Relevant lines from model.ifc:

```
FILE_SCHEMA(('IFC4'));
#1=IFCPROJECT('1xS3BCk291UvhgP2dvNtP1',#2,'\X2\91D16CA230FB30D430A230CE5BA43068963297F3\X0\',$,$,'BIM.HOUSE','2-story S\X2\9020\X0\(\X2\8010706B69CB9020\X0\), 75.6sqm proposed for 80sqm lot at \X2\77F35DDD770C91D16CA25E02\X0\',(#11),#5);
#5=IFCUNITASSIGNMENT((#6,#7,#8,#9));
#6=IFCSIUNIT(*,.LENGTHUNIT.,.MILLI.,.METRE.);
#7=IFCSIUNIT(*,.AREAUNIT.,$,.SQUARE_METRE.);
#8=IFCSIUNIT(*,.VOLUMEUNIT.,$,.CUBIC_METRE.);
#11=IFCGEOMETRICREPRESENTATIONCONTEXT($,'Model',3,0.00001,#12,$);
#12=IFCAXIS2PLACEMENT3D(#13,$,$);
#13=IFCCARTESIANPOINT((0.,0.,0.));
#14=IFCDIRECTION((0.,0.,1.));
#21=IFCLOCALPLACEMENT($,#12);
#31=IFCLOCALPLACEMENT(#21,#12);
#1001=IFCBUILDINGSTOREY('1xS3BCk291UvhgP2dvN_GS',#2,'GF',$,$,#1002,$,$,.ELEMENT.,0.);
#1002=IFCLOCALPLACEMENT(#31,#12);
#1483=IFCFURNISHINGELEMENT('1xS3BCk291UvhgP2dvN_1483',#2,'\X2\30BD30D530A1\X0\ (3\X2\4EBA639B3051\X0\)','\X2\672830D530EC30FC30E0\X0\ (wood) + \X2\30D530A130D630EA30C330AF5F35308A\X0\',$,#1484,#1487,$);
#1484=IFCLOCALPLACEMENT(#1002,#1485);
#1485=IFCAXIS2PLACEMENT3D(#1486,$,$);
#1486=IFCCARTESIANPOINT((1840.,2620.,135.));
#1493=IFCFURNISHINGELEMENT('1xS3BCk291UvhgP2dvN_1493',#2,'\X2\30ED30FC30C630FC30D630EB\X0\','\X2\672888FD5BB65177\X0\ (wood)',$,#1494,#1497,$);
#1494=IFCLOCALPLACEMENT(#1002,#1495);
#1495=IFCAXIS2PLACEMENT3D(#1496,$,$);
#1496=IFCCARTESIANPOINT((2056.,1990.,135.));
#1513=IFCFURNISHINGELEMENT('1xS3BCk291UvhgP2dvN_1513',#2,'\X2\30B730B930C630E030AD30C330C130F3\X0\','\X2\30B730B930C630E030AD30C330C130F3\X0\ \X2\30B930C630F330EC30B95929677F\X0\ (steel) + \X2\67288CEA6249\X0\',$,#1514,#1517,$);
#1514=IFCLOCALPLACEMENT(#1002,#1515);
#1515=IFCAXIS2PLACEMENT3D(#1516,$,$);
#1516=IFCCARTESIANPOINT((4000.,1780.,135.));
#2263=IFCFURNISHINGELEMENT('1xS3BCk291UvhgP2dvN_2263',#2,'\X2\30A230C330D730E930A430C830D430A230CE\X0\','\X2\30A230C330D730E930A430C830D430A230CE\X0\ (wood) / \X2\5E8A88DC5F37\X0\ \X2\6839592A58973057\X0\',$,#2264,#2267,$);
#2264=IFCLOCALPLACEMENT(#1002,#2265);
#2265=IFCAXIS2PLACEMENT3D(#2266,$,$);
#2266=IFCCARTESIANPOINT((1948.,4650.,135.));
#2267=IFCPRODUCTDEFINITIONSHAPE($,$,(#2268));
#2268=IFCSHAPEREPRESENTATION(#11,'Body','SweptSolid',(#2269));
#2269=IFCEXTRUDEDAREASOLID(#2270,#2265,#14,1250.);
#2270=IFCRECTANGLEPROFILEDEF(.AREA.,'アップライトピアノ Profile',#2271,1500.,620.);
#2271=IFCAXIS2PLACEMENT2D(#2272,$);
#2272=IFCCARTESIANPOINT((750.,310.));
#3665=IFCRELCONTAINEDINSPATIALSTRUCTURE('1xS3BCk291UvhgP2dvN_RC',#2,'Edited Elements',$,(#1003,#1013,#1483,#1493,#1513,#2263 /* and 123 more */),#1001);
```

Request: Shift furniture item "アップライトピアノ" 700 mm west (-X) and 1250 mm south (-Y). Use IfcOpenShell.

```python
import ifcopenshell
import ifcopenshell.api.geometry
import ifcopenshell.util.placement

model = ifcopenshell.open("model.ifc")

item = model.by_guid("1xS3BCk291UvhgP2dvN_2263")
matrix = ifcopenshell.util.placement.get_local_placement(item.ObjectPlacement)
matrix[0, 3] -= 700.0
matrix[1, 3] -= 1250.0
ifcopenshell.api.geometry.edit_object_placement(model, product=item, matrix=matrix, is_si=False)

print(ifcopenshell.util.placement.get_local_placement(item.ObjectPlacement).round(3) + 0.0)

model.write("model-out.ifc")
```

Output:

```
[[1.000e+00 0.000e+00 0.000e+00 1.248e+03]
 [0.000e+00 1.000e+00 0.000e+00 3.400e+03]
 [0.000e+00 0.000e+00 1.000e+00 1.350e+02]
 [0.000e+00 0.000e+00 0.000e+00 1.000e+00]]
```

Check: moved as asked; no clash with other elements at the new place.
